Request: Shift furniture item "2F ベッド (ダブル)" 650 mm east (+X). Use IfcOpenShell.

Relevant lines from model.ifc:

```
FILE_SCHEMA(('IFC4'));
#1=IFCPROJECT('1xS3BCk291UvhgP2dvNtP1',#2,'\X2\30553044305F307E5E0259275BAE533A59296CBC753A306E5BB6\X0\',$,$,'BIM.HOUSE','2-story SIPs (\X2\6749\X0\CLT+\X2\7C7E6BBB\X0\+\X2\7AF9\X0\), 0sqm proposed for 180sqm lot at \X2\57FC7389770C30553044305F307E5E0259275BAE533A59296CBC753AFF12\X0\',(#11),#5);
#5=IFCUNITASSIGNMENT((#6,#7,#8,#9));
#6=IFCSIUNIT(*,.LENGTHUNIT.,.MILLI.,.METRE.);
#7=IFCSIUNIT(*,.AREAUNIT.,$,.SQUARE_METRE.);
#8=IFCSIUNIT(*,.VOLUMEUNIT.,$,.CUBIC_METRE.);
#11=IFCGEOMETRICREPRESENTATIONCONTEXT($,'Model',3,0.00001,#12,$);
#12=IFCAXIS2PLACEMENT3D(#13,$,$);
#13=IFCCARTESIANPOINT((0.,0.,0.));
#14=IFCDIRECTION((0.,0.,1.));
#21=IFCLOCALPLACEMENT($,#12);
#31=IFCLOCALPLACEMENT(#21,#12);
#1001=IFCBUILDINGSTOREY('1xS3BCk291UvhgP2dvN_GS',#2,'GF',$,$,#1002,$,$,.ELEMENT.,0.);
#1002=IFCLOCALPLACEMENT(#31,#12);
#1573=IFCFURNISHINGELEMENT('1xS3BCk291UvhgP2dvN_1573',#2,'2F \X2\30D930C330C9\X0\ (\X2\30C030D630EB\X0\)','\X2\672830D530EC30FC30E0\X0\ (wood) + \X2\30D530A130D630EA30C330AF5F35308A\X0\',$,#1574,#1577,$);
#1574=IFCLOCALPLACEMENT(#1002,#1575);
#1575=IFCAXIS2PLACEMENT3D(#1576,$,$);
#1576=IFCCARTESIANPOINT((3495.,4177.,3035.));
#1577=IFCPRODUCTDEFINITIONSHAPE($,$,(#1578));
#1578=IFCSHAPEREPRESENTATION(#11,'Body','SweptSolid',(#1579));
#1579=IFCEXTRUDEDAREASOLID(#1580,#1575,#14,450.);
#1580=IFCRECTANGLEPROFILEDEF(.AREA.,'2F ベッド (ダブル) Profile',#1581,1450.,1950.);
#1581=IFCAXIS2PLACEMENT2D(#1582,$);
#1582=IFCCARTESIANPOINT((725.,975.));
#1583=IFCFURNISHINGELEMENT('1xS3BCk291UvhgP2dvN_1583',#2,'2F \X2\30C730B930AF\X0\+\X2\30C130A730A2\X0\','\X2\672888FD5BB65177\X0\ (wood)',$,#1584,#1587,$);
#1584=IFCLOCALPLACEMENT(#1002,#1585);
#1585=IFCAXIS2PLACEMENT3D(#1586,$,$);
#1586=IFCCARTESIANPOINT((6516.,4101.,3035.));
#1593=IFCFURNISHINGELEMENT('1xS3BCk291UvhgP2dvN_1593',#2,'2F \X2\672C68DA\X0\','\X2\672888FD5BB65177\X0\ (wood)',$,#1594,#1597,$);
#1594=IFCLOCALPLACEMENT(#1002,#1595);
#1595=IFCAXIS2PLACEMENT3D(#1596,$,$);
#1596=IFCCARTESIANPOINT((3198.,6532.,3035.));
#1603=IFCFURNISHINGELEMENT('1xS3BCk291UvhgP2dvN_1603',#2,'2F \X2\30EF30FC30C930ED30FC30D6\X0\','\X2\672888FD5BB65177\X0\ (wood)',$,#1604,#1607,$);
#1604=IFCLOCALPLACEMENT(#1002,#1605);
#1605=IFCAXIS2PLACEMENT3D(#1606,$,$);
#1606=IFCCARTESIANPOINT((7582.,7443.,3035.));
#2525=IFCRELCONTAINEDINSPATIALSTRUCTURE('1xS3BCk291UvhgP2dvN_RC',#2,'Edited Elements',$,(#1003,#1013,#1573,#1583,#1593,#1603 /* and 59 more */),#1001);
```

```python
import ifcopenshell
import ifcopenshell.api.geometry
import ifcopenshell.util.placement
import ifcopenshell.util.unit

model = ifcopenshell.open("model.ifc")
unit_scale = ifcopenshell.util.unit.calculate_unit_scale(model)

item = model.by_guid("1xS3BCk291UvhgP2dvN_1573")
matrix = ifcopenshell.util.placement.get_local_placement(item.ObjectPlacement)
matrix[0, 3] += 0.65 / unit_scale
ifcopenshell.api.geometry.edit_object_placement(model, product=item, matrix=matrix, is_si=False)

print(ifcopenshell.util.placement.get_local_placement(item.ObjectPlacement).round(3) + 0.0)

model.write("model_updated.ifc")
```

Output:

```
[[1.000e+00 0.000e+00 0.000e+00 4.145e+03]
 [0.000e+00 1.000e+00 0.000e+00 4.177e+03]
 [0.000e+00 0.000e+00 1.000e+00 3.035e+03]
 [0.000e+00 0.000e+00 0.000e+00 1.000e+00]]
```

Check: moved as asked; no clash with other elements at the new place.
